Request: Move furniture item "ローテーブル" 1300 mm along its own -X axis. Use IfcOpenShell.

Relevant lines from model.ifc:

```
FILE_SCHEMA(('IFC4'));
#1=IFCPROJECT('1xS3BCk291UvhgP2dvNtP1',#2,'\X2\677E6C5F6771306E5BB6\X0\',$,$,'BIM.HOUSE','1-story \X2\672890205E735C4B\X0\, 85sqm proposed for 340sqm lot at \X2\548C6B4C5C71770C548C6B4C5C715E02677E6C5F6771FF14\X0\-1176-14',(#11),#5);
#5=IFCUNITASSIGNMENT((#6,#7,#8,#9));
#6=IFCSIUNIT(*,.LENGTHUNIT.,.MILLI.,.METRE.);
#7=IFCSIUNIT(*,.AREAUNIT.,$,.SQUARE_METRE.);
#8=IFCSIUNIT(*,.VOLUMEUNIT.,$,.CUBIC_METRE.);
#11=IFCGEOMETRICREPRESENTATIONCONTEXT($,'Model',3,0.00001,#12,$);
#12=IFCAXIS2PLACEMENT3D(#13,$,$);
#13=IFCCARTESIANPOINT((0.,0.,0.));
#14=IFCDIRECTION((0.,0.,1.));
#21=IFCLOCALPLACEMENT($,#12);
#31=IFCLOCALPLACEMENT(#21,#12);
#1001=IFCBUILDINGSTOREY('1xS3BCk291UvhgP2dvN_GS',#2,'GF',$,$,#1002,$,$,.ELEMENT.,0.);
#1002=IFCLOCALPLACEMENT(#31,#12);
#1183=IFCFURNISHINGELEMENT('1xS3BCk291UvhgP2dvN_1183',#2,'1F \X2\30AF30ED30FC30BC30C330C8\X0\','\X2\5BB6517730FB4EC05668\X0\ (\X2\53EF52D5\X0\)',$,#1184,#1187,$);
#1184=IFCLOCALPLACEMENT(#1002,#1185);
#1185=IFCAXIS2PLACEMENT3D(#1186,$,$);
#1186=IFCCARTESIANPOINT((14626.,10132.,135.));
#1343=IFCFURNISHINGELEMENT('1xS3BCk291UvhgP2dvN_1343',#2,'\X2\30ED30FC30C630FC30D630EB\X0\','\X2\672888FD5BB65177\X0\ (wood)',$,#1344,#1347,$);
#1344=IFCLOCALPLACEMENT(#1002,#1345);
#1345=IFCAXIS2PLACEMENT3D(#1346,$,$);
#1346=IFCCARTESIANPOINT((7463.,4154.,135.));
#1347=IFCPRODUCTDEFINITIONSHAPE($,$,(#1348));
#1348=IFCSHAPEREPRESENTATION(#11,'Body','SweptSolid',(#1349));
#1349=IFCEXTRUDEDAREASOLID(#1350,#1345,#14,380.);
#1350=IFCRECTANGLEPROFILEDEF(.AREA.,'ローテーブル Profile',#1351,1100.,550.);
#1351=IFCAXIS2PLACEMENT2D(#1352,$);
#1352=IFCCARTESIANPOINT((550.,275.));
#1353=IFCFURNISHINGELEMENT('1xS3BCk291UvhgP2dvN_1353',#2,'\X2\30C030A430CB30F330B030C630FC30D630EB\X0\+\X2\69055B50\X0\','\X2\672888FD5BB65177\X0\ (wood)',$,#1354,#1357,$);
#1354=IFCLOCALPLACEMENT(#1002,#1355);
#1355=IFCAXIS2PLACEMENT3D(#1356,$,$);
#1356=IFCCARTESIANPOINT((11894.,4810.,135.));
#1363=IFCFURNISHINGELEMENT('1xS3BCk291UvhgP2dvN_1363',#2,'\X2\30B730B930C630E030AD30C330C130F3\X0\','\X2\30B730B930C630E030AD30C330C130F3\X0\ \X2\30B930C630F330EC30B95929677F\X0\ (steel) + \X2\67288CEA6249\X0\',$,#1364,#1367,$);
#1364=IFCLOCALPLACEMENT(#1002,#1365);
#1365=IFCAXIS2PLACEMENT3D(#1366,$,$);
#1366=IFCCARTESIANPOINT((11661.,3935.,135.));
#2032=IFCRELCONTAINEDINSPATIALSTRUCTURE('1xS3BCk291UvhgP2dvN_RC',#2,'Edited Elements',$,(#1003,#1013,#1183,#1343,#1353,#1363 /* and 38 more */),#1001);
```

```python
import ifcopenshell
import ifcopenshell.api.geometry
import ifcopenshell.util.placement
import ifcopenshell.util.unit

model = ifcopenshell.open("model.ifc")
unit_scale = ifcopenshell.util.unit.calculate_unit_scale(model)

item = model.by_id(1343)
matrix = ifcopenshell.util.placement.get_local_placement(item.ObjectPlacement)
matrix[:3, 3] -= matrix[:3, 0] * 1.3 / unit_scale
ifcopenshell.api.geometry.edit_object_placement(model, product=item, matrix=matrix, is_si=False)

print(ifcopenshell.util.placement.get_local_placement(item.ObjectPlacement).round(3) + 0.0)

model.write("model_updated.ifc")
```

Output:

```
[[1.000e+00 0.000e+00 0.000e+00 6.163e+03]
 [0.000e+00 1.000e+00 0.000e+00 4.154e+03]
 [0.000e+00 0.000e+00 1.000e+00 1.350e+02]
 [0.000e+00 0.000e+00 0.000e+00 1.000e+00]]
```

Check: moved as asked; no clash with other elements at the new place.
